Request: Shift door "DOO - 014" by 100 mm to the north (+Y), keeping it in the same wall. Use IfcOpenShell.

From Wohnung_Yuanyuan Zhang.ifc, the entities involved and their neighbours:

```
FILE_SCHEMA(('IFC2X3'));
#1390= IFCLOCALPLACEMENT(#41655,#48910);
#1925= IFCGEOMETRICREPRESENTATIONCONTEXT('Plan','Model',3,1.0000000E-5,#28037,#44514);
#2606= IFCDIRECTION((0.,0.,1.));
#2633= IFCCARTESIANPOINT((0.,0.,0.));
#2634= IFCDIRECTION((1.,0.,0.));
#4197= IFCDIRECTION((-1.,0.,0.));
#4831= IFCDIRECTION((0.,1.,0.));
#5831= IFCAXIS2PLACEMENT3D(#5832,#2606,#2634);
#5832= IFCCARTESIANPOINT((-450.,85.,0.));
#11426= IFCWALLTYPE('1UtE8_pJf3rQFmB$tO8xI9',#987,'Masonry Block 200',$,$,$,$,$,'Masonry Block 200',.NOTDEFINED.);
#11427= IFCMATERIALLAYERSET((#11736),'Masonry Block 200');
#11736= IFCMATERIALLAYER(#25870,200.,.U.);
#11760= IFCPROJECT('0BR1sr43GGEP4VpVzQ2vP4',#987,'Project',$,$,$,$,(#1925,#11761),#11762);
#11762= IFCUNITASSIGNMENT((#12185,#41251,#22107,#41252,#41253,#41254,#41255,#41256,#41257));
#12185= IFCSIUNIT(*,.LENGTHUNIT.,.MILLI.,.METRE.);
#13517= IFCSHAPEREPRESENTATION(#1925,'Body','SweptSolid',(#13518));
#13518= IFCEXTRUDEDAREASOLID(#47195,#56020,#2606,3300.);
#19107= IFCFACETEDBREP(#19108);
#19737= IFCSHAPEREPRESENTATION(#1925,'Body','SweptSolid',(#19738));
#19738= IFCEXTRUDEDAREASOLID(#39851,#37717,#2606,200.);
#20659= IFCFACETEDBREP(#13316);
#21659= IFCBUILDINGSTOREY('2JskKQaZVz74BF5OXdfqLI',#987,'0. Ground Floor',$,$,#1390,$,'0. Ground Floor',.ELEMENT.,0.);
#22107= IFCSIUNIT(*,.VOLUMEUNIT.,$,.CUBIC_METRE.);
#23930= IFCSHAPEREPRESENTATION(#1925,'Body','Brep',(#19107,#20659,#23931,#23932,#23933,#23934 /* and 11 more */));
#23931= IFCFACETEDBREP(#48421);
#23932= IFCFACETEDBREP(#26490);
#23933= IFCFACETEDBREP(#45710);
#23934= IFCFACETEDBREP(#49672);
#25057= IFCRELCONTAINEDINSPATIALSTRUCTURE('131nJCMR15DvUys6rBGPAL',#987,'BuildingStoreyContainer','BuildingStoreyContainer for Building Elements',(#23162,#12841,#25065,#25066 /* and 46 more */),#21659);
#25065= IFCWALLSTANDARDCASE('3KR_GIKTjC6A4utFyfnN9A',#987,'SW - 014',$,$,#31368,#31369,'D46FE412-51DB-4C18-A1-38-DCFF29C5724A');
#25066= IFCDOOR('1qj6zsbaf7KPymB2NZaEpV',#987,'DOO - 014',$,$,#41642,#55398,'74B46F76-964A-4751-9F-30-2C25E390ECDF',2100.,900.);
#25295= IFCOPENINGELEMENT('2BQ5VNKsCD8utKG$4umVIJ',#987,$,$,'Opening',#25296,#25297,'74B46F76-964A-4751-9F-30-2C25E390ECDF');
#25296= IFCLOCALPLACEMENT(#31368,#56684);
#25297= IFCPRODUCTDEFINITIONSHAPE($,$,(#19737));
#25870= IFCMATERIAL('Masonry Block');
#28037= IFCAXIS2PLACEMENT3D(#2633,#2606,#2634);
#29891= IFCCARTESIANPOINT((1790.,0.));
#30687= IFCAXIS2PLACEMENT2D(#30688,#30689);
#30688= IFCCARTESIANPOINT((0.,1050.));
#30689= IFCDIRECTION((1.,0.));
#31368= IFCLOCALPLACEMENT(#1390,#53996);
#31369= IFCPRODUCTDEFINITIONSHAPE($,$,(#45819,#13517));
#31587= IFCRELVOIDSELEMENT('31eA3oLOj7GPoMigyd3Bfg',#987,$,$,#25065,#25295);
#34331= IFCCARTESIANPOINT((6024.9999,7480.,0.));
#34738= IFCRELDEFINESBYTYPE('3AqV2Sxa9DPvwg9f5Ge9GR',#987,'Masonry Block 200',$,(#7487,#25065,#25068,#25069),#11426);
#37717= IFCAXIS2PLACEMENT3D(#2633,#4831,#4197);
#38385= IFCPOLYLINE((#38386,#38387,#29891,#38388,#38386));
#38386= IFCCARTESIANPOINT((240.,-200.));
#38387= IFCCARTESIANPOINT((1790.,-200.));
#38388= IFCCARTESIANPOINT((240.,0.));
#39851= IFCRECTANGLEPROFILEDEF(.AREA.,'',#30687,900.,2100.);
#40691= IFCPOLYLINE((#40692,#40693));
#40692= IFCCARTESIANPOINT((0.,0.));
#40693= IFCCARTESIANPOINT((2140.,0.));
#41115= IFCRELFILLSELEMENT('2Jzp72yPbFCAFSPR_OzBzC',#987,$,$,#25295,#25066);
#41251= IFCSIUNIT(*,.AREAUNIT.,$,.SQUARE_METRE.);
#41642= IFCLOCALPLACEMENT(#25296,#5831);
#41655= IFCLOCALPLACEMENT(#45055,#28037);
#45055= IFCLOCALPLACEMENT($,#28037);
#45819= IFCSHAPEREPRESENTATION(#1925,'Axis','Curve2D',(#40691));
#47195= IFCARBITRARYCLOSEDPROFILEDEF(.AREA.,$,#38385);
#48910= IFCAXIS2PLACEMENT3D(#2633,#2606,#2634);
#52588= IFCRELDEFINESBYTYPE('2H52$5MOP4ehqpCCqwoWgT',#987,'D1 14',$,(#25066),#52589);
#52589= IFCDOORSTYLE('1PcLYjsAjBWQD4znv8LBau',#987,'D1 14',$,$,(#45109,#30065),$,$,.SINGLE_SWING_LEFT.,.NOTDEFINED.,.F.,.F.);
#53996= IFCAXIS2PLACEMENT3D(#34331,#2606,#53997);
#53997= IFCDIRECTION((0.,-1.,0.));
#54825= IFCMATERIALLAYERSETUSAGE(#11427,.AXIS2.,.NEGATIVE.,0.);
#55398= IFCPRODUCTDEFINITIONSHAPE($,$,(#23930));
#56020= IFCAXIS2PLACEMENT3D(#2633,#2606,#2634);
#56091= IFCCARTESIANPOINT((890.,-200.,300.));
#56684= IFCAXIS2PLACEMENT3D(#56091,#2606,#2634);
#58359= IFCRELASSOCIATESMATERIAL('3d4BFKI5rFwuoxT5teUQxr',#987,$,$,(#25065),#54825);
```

```python
import ifcopenshell
import ifcopenshell.api.geometry
import ifcopenshell.util.placement

model = ifcopenshell.open("Wohnung_Yuanyuan Zhang.ifc")

door = model.by_id(25066)
opening = door.FillsVoids[0].RelatingOpeningElement
wall = opening.VoidsElements[0].RelatingBuildingElement

wall_matrix = ifcopenshell.util.placement.get_local_placement(wall.ObjectPlacement)
shift = wall_matrix[:3, 0] * -100.0
before = ifcopenshell.util.placement.get_local_placement(door.ObjectPlacement)[:3, 3].copy()

# The door is placed relative to its opening, so it follows when the opening moves.
matrix = ifcopenshell.util.placement.get_local_placement(opening.ObjectPlacement)
matrix[:3, 3] += shift
ifcopenshell.api.geometry.edit_object_placement(
    model, product=opening, matrix=matrix, is_si=False, should_transform_children=True
)

after = ifcopenshell.util.placement.get_local_placement(door.ObjectPlacement)[:3, 3]
print("door moved by", (after - before).round(3) + 0.0)

model.write("Wohnung_Yuanyuan Zhang_rev.ifc")
```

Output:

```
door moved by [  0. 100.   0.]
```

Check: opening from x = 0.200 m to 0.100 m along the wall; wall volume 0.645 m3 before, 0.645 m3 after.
